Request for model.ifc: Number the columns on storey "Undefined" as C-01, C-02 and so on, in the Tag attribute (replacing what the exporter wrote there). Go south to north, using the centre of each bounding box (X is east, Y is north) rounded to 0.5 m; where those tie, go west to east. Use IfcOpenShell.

First a look at what the model holds.

```python
import ifcopenshell
import ifcopenshell.util.element
import ifcopenshell.util.placement

model = ifcopenshell.open("model.ifc")
print(model.schema)
storey = next(s for s in model.by_type("IfcBuildingStorey") if s.Name == "Undefined")
columns = [e for e in ifcopenshell.util.element.get_decomposition(storey) if e.is_a("IfcColumn")]
for e in sorted(columns, key=lambda e: e.id()):
    origin = ifcopenshell.util.placement.get_local_placement(e.ObjectPlacement)[:3, 3]
    print(e.id(), e.Tag, e.Name, origin.round(2) + 0.0, sep=" | ")
```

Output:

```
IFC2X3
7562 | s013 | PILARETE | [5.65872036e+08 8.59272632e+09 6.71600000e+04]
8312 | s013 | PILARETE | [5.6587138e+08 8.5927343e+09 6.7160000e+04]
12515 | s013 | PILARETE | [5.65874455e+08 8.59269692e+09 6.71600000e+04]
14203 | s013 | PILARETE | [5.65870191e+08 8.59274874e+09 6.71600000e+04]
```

```python
import ifcopenshell
import ifcopenshell.geom
import ifcopenshell.util.element
import ifcopenshell.util.shape

model = ifcopenshell.open("model.ifc")
settings = ifcopenshell.geom.settings()
settings.set("use-world-coords", True)


def centre(element):
    shape = ifcopenshell.geom.create_shape(settings, element)
    return ifcopenshell.util.shape.get_bbox_centroid(shape.geometry)


storey = next(s for s in model.by_type("IfcBuildingStorey") if s.Name == "Undefined")
columns = [e for e in ifcopenshell.util.element.get_decomposition(storey) if e.is_a("IfcColumn")]

# Insertion points can sit at a corner or the storey origin, so sort by the geometry (in metres).
centres = {e: centre(e) for e in columns}
columns.sort(key=lambda e: (round(centres[e][1] / 0.5), centres[e][0]))

for i, e in enumerate(columns, start=1):
    number = f"C-{i:02d}"
    e.Tag = number
    print(e.id(), number)

model.write("model-out.ifc")
```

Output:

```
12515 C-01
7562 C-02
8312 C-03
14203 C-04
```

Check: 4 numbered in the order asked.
